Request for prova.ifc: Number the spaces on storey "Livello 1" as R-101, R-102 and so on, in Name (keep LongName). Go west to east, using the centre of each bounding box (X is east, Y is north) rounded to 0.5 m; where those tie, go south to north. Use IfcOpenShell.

First a look at what the model holds.

```python
import ifcopenshell
import ifcopenshell.util.element
import ifcopenshell.util.placement

model = ifcopenshell.open("prova.ifc")
print(model.schema)
storey = next(s for s in model.by_type("IfcBuildingStorey") if s.Name == "Livello 1")
spaces = [e for e in ifcopenshell.util.element.get_decomposition(storey) if e.is_a("IfcSpace")]
for e in sorted(spaces, key=lambda e: e.id()):
    origin = ifcopenshell.util.placement.get_local_placement(e.ObjectPlacement)[:3, 3]
    print(e.id(), e.Name, e.LongName, origin.round(2) + 0.0, sep=" | ")
```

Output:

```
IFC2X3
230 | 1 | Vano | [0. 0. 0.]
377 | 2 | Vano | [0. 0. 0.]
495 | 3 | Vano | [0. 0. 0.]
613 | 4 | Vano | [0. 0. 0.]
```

```python
import ifcopenshell
import ifcopenshell.geom
import ifcopenshell.util.element
import ifcopenshell.util.shape

model = ifcopenshell.open("prova.ifc")
settings = ifcopenshell.geom.settings()
settings.set("use-world-coords", True)


def centre(element):
    shape = ifcopenshell.geom.create_shape(settings, element)
    return ifcopenshell.util.shape.get_bbox_centroid(shape.geometry)


storey = next(s for s in model.by_type("IfcBuildingStorey") if s.Name == "Livello 1")
spaces = [e for e in ifcopenshell.util.element.get_decomposition(storey) if e.is_a("IfcSpace")]

# Insertion points can sit at a corner or the storey origin, so sort by the geometry (in metres).
centres = {e: centre(e) for e in spaces}
spaces.sort(key=lambda e: (round(centres[e][0] / 0.5), centres[e][1]))

for i, e in enumerate(spaces, start=1):
    number = f"R-1{i:02d}"
    e.Name = number
    print(e.id(), number)

model.write("prova_v2.ifc")
```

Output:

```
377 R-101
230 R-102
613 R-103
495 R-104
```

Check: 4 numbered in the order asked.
